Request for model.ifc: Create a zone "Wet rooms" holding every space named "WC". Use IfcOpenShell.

First a look at what the model holds.

```python
import ifcopenshell

model = ifcopenshell.open("model.ifc")
print(model.schema)
seen = {}
for space in model.by_type("IfcSpace"):
    seen[space.LongName] = seen.get(space.LongName, 0) + 1
for name, count in sorted(seen.items(), key=str):
    print(count, "x", name)
print("zones:", [z.Name for z in model.by_type("IfcZone")][:20])
```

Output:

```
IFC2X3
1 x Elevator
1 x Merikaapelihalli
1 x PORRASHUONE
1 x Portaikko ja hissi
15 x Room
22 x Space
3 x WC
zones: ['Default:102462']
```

```python
import ifcopenshell
import ifcopenshell.api.group
import ifcopenshell.api.root

model = ifcopenshell.open("model.ifc")

names = {"WC"}
spaces = [s for s in model.by_type("IfcSpace") if s.LongName in names]

zone = ifcopenshell.api.root.create_entity(model, ifc_class="IfcZone", name="Wet rooms")
ifcopenshell.api.group.assign_group(model, products=spaces, group=zone)
print(len(spaces), "spaces in", zone.Name)

model.write("model_v2.ifc")
```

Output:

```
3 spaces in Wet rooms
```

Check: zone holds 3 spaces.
